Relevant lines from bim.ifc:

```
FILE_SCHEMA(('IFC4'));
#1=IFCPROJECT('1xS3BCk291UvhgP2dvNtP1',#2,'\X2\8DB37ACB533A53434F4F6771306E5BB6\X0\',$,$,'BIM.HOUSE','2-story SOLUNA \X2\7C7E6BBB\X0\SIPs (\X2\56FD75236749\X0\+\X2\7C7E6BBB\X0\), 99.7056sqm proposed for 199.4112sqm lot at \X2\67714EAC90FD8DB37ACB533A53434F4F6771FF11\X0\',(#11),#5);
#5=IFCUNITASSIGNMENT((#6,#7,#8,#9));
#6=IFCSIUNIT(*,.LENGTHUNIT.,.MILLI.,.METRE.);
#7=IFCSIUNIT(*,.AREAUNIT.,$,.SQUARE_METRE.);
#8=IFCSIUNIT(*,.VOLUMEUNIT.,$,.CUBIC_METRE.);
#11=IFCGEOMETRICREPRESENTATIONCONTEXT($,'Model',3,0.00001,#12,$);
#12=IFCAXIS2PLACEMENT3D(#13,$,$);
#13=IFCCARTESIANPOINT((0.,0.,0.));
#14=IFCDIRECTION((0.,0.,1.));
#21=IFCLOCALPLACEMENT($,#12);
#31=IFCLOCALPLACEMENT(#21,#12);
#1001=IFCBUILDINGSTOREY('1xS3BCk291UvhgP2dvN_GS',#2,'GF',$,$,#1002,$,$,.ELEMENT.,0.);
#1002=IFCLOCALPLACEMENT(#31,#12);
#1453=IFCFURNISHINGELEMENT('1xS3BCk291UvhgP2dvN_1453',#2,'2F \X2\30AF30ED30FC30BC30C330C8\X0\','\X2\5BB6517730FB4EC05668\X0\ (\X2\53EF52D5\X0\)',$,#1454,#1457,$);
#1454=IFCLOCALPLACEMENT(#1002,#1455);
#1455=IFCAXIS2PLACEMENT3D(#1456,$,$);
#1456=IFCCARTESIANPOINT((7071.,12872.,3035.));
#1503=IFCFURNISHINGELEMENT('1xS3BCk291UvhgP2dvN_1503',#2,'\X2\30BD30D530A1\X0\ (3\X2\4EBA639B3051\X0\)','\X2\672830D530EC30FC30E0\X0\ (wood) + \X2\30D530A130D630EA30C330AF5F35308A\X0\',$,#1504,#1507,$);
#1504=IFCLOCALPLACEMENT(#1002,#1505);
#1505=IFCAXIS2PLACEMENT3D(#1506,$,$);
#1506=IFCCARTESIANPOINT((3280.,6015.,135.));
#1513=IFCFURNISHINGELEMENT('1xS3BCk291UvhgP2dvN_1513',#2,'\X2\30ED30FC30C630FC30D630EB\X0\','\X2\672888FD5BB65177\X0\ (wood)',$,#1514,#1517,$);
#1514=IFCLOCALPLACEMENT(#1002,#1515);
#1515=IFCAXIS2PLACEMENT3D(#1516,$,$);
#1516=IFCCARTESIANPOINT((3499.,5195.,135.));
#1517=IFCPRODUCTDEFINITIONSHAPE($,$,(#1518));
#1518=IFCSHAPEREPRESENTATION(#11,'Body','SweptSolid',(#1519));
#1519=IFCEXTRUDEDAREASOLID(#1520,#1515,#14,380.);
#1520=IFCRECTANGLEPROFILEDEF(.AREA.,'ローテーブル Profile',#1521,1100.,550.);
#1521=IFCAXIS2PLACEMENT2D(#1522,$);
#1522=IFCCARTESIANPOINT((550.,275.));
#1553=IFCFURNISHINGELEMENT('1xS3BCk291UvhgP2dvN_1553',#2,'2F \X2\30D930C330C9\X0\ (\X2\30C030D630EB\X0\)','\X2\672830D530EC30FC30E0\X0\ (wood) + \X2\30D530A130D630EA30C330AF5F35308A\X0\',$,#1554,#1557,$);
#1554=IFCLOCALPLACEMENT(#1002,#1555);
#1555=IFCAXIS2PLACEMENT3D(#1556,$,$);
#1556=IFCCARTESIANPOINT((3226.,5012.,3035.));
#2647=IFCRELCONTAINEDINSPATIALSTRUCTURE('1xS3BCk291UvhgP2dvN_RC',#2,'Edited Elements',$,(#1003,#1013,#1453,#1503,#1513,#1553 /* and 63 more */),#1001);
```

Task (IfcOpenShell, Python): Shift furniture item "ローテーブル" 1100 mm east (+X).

```python
import ifcopenshell
import ifcopenshell.api.geometry
import ifcopenshell.util.placement
import ifcopenshell.util.unit

model = ifcopenshell.open("bim.ifc")
unit_scale = ifcopenshell.util.unit.calculate_unit_scale(model)

item = model.by_guid("1xS3BCk291UvhgP2dvN_1513")
matrix = ifcopenshell.util.placement.get_local_placement(item.ObjectPlacement)
matrix[0, 3] += 1.1 / unit_scale
ifcopenshell.api.geometry.edit_object_placement(model, product=item, matrix=matrix, is_si=False)

print(ifcopenshell.util.placement.get_local_placement(item.ObjectPlacement).round(3) + 0.0)

model.write("bim_rev.ifc")
```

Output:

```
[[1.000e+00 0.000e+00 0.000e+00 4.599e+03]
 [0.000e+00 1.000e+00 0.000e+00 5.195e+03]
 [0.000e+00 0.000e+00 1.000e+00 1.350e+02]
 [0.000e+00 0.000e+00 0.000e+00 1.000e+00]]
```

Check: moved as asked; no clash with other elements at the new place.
